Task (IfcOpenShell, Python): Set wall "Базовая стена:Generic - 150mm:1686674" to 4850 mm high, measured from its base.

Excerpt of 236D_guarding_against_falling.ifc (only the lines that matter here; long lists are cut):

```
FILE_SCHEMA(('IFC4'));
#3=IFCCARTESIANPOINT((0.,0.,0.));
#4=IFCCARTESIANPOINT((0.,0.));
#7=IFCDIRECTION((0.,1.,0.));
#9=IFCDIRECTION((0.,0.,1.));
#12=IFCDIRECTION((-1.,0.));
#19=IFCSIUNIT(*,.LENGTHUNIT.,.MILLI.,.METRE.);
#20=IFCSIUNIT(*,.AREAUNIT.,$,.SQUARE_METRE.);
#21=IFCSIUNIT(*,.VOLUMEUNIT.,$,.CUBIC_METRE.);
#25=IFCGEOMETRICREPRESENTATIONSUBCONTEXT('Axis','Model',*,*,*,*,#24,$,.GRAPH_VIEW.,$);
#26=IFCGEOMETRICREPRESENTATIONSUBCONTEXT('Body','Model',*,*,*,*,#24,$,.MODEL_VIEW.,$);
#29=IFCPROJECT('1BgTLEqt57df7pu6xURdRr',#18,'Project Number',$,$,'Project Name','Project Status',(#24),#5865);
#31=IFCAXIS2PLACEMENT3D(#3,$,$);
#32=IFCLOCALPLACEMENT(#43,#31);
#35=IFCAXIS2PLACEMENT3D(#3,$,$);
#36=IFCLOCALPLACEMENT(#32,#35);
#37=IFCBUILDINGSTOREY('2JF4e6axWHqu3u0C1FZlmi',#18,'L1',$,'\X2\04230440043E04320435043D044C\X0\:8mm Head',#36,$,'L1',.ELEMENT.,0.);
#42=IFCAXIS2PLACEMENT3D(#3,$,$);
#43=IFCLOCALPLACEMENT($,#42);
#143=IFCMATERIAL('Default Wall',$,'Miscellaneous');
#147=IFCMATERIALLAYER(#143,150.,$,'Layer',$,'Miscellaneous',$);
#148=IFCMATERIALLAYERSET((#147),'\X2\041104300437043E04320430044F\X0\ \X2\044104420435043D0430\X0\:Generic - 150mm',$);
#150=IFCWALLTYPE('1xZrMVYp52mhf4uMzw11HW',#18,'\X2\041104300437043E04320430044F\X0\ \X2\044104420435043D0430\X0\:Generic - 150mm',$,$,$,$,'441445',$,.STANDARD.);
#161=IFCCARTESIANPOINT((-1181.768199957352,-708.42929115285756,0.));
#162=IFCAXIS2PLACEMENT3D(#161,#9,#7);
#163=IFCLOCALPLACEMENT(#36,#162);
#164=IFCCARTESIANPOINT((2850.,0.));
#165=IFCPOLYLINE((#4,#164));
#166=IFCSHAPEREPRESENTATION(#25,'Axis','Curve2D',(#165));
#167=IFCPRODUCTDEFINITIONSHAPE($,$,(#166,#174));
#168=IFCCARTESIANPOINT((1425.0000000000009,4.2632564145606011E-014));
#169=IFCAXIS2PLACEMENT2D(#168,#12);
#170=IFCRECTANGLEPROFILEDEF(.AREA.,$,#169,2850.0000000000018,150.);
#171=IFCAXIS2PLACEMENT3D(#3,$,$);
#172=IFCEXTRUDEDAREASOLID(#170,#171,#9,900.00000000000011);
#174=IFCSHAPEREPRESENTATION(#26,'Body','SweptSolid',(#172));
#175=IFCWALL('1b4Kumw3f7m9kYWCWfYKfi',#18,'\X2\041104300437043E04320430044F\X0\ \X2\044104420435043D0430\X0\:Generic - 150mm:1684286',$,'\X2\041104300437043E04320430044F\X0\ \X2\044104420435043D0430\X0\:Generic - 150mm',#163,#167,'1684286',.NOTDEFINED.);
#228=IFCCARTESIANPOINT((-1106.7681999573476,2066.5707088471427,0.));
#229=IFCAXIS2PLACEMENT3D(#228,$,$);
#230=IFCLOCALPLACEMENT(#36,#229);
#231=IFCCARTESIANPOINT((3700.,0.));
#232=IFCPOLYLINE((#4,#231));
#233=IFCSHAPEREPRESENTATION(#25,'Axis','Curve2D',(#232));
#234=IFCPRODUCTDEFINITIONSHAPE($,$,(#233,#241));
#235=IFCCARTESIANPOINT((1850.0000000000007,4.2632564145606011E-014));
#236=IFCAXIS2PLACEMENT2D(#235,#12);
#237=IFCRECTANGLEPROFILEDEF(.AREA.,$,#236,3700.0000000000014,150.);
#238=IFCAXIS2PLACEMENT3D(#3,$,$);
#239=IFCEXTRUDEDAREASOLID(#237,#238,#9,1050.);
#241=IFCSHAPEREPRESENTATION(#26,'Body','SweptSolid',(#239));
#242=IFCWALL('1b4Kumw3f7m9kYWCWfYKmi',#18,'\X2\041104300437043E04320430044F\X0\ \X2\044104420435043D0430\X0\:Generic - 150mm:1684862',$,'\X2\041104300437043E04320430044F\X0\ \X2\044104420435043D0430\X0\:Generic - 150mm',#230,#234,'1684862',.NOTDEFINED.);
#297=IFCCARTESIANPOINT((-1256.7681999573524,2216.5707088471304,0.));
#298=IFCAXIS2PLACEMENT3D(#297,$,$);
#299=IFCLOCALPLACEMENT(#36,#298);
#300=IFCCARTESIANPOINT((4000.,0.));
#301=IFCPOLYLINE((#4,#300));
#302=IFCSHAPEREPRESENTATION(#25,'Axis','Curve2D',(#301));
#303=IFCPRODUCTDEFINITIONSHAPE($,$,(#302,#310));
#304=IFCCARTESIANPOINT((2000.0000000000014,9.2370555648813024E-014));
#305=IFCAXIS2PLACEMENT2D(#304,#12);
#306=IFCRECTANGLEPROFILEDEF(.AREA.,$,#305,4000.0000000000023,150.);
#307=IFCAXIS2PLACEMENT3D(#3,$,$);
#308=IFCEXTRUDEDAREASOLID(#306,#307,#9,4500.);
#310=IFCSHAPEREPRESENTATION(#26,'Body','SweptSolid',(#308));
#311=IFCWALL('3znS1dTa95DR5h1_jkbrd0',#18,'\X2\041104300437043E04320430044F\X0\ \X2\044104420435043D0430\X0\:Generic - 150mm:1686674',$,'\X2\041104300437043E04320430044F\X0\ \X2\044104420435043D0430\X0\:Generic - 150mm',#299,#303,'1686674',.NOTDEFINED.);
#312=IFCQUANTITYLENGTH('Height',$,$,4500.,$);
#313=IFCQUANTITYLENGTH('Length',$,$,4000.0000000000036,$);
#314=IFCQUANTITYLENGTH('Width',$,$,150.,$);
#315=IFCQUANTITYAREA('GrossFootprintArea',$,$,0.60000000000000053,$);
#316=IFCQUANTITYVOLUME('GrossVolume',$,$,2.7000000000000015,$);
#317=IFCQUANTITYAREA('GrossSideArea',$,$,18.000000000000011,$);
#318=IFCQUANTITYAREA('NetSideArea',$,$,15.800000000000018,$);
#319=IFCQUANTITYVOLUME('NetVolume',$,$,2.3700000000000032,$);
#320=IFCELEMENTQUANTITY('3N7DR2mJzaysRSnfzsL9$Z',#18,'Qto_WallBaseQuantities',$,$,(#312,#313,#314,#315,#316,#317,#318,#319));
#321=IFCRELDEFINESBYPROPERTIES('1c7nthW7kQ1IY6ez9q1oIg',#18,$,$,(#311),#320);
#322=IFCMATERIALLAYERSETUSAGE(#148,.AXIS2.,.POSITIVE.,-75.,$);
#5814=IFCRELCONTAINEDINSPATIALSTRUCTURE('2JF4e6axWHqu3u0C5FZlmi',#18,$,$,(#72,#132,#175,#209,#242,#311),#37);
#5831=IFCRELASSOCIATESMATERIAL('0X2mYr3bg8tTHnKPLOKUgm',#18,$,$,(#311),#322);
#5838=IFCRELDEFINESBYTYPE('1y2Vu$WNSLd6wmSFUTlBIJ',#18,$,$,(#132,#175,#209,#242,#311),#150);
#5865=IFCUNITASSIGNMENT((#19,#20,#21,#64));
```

```python
import ifcopenshell
import ifcopenshell.api.pset
import ifcopenshell.geom
import ifcopenshell.util.element
import ifcopenshell.util.representation
import ifcopenshell.util.shape
import ifcopenshell.util.unit

model = ifcopenshell.open("236D_guarding_against_falling.ifc")
unit_scale = ifcopenshell.util.unit.calculate_unit_scale(model)
area_scale = ifcopenshell.util.unit.calculate_unit_scale(model, "AREAUNIT")
volume_scale = ifcopenshell.util.unit.calculate_unit_scale(model, "VOLUMEUNIT")
settings = ifcopenshell.geom.settings()


def volume(element):
    """Net volume in cubic metres, openings subtracted."""
    shape = ifcopenshell.geom.create_shape(settings, element)
    return ifcopenshell.util.shape.get_volume(shape.geometry)


wall = model.by_guid("3znS1dTa95DR5h1_jkbrd0")
before = volume(wall)

body = ifcopenshell.util.representation.get_representation(wall, "Model", "Body")
solid = body.Items[0]
old_height = solid.Depth
solid.Depth = 4.85 / unit_scale
after = volume(wall)
thickness = 0.15  # wall thickness in metres

# Update the stored height, areas and volumes.
qto = model.by_id(ifcopenshell.util.element.get_pset(wall, "Qto_WallBaseQuantities", should_inherit=False)["id"])
ifcopenshell.api.pset.edit_qto(model, qto=qto, properties={
    "Height": solid.Depth,
    "GrossVolume": ifcopenshell.util.element.get_pset(wall, "Qto_WallBaseQuantities", "GrossVolume") * solid.Depth / old_height,
    "GrossSideArea": ifcopenshell.util.element.get_pset(wall, "Qto_WallBaseQuantities", "GrossSideArea") * solid.Depth / old_height,
    "NetSideArea": after / thickness / area_scale,
    "NetVolume": after / volume_scale,
})

print(f"height {old_height:g} -> {solid.Depth:g}, volume {before:.3f} -> {after:.3f} m3")

model.write("236D_guarding_against_falling_rev.ifc")
```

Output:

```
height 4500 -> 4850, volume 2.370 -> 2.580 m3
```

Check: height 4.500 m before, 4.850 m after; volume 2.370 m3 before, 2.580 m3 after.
